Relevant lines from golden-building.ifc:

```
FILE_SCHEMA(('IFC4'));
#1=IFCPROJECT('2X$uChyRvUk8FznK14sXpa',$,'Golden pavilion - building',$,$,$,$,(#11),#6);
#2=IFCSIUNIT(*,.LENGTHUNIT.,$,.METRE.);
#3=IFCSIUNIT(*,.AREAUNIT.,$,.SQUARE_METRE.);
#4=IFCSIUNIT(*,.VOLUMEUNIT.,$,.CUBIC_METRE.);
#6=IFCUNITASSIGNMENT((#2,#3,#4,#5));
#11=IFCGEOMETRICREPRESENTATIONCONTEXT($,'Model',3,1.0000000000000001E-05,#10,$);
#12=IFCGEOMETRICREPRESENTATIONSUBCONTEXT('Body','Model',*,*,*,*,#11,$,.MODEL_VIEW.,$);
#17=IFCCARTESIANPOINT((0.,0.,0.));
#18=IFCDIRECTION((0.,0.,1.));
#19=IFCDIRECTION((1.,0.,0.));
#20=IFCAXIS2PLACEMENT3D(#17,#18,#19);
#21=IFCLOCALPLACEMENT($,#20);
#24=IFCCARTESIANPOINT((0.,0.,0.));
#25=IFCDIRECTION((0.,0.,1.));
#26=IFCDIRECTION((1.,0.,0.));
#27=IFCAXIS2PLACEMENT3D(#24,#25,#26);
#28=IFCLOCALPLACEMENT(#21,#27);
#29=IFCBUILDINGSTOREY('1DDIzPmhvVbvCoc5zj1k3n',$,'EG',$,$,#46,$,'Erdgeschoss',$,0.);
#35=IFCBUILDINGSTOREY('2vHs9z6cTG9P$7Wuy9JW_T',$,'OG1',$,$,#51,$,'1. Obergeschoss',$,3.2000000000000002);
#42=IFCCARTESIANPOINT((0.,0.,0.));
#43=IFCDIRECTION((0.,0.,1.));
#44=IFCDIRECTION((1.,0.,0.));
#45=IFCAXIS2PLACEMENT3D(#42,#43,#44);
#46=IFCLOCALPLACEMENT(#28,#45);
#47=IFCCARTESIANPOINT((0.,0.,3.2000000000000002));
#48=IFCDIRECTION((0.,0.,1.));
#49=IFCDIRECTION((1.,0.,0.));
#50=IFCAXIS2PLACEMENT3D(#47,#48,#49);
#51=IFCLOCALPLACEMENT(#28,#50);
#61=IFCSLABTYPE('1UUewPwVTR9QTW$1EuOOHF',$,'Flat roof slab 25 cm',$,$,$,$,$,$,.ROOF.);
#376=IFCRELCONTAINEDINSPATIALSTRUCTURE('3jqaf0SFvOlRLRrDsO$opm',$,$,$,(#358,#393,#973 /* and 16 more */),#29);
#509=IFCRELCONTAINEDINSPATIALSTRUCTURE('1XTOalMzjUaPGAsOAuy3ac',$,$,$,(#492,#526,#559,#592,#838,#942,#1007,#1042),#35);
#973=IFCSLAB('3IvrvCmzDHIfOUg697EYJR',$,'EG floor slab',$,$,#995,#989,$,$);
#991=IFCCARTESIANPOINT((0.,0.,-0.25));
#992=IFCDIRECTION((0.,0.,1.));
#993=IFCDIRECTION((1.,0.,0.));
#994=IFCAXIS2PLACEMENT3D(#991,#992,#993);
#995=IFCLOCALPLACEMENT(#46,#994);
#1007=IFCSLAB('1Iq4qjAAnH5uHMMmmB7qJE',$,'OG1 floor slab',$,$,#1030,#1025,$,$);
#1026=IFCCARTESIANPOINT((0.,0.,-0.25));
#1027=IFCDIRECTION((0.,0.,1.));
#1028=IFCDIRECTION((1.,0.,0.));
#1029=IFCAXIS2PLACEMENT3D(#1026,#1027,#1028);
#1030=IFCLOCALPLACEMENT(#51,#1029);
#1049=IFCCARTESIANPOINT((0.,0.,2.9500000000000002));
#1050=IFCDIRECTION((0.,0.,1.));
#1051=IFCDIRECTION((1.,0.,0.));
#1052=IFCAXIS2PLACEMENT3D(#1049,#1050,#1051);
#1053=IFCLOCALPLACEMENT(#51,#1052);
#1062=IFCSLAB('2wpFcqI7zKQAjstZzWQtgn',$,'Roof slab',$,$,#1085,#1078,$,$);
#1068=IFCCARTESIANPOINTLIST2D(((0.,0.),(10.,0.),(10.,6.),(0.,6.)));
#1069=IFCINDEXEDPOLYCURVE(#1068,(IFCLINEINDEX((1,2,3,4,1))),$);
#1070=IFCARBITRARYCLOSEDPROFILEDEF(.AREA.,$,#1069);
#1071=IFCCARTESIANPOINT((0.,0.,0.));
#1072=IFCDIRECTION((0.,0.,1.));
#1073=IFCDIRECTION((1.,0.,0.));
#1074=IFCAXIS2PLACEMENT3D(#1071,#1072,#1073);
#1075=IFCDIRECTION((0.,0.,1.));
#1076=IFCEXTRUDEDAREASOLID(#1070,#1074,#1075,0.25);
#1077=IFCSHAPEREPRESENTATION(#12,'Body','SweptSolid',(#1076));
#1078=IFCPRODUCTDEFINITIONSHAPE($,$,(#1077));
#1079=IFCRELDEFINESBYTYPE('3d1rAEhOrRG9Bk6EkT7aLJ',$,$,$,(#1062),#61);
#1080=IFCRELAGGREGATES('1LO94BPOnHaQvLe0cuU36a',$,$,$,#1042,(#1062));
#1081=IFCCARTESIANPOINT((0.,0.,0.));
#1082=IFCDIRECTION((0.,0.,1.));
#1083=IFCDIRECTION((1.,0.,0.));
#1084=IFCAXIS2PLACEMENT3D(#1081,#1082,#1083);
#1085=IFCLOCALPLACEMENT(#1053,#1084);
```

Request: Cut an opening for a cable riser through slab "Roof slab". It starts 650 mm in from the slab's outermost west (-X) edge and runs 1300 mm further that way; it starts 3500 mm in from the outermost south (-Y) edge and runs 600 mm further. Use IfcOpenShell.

```python
import numpy as np
import ifcopenshell
import ifcopenshell.api.feature
import ifcopenshell.api.geometry
import ifcopenshell.api.root
import ifcopenshell.geom
import ifcopenshell.util.placement
import ifcopenshell.util.representation
import ifcopenshell.util.shape
import ifcopenshell.util.unit

model = ifcopenshell.open("golden-building.ifc")
unit_scale = ifcopenshell.util.unit.calculate_unit_scale(model)
settings = ifcopenshell.geom.settings()


def volume(element):
    """Net volume in cubic metres, openings subtracted."""
    shape = ifcopenshell.geom.create_shape(settings, element)
    return ifcopenshell.util.shape.get_volume(shape.geometry)


slab = model.by_guid("2wpFcqI7zKQAjstZzWQtgn")
before = volume(slab)

# Extent in the slab's own axes, in metres. The edges named are its -X and -Y sides.
slab_shape = ifcopenshell.geom.create_shape(settings, slab)
vertices = ifcopenshell.util.shape.get_vertices(slab_shape.geometry)
x_min, y_min, bottom = vertices.min(axis=0)
top = vertices[:, 2].max()

opening = ifcopenshell.api.root.create_entity(model, ifc_class="IfcOpeningElement", name="Cable riser opening", predefined_type="OPENING")
context = ifcopenshell.util.representation.get_context(model, "Model", "Body", "MODEL_VIEW")
width, depth = 1.3, 0.6
outline = [(0.0, 0.0), (width, 0.0), (width, depth), (0.0, depth), (0.0, 0.0)]
# Overshoot both faces by 50 mm so the cut is clean.
shape = ifcopenshell.api.geometry.add_slab_representation(
    model, context=context, depth=top - bottom + 0.1, polyline=outline
)
ifcopenshell.api.geometry.assign_representation(model, product=opening, representation=shape)

matrix = ifcopenshell.util.placement.get_local_placement(slab.ObjectPlacement)
matrix[:, 3] = matrix @ np.append(np.array([x_min + 0.65, y_min + 3.5, bottom - 0.05]) / unit_scale, 1.0)
ifcopenshell.api.geometry.edit_object_placement(model, product=opening, matrix=matrix, is_si=False)
ifcopenshell.api.feature.add_feature(model, feature=opening, element=slab)

after = volume(slab)

print(f"slab volume {before:.3f} -> {after:.3f} m3")

model.write("golden-building_updated.ifc")
```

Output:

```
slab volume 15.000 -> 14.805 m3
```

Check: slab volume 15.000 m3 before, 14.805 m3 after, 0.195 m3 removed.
